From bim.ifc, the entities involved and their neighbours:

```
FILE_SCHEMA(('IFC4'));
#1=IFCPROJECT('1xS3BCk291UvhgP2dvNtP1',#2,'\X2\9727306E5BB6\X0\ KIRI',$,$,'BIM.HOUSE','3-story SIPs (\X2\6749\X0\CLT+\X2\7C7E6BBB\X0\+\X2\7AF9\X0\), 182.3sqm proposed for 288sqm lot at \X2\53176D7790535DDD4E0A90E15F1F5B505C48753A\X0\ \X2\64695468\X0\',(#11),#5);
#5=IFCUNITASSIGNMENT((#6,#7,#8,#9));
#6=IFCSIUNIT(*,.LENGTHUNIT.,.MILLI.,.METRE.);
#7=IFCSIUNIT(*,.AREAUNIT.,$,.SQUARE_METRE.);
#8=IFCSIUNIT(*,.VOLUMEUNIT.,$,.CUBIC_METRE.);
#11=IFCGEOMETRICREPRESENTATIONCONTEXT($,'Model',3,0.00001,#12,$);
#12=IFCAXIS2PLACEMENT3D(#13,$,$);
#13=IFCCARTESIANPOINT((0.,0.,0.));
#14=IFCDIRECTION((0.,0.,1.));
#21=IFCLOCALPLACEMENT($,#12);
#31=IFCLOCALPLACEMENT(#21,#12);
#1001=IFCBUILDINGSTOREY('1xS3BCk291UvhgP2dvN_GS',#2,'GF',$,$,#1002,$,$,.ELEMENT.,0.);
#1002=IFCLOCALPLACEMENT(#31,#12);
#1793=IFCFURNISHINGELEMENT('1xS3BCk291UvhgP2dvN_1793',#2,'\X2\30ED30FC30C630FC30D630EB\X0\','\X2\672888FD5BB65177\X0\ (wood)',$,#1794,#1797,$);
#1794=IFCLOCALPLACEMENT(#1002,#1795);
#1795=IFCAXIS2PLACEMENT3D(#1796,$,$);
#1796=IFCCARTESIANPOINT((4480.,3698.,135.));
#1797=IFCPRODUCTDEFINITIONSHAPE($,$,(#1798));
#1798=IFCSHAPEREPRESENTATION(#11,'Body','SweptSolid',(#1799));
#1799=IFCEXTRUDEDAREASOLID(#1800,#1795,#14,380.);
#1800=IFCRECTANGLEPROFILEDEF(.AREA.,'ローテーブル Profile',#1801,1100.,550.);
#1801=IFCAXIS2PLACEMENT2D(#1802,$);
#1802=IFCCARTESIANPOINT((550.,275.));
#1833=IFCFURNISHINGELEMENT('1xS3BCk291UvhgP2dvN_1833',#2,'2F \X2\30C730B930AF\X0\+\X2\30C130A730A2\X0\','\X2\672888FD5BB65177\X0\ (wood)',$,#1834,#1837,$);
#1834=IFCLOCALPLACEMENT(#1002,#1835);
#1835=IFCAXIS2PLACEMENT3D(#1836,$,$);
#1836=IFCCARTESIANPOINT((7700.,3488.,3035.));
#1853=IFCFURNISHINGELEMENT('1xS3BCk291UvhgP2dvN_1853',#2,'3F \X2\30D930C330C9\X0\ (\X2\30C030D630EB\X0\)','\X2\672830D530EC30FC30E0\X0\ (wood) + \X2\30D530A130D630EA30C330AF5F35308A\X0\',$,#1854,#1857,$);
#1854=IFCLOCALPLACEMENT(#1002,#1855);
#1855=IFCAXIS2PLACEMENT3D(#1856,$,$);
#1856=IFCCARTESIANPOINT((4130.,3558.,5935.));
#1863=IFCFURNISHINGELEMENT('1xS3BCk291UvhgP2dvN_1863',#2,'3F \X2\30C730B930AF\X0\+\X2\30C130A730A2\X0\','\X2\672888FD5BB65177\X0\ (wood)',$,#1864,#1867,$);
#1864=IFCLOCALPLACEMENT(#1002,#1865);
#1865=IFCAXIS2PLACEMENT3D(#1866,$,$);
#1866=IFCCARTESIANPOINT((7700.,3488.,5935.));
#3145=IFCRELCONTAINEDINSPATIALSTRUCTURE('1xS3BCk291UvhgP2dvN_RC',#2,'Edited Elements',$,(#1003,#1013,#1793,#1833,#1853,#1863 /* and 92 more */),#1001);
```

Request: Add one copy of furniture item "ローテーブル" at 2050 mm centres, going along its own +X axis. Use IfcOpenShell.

```python
import ifcopenshell
import ifcopenshell.api.geometry
import ifcopenshell.api.root
import ifcopenshell.util.element
import ifcopenshell.util.placement

model = ifcopenshell.open("bim.ifc")


def reuse_history(source, copy):
    """copy_class also copies each property set's owner history, people and application; keep the originals."""
    for rel in copy.IsDefinedBy:
        if rel.is_a("IfcRelDefinesByProperties") and (history := rel.RelatingPropertyDefinition.OwnerHistory):
            rel.RelatingPropertyDefinition.OwnerHistory = source.OwnerHistory
            ifcopenshell.util.element.remove_deep2(model, history)


source = model.by_id(1793)
base = ifcopenshell.util.placement.get_local_placement(source.ObjectPlacement)
step = base[:3, 0] * 2050.0

for i in range(1, 2):
    copy = ifcopenshell.api.root.copy_class(model, product=source)
    copy.Representation = ifcopenshell.util.element.copy_deep(
        model, source.Representation, exclude=["IfcGeometricRepresentationContext", "IfcRepresentationMap"]
    )
    reuse_history(source, copy)
    matrix = base.copy()
    matrix[:3, 3] += i * step
    print("added at", matrix[:3, 3].round(3) + 0.0)
    ifcopenshell.api.geometry.edit_object_placement(model, product=copy, matrix=matrix, is_si=False)

model.write("bim_edited.ifc")
```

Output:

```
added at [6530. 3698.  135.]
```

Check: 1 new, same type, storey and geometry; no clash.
